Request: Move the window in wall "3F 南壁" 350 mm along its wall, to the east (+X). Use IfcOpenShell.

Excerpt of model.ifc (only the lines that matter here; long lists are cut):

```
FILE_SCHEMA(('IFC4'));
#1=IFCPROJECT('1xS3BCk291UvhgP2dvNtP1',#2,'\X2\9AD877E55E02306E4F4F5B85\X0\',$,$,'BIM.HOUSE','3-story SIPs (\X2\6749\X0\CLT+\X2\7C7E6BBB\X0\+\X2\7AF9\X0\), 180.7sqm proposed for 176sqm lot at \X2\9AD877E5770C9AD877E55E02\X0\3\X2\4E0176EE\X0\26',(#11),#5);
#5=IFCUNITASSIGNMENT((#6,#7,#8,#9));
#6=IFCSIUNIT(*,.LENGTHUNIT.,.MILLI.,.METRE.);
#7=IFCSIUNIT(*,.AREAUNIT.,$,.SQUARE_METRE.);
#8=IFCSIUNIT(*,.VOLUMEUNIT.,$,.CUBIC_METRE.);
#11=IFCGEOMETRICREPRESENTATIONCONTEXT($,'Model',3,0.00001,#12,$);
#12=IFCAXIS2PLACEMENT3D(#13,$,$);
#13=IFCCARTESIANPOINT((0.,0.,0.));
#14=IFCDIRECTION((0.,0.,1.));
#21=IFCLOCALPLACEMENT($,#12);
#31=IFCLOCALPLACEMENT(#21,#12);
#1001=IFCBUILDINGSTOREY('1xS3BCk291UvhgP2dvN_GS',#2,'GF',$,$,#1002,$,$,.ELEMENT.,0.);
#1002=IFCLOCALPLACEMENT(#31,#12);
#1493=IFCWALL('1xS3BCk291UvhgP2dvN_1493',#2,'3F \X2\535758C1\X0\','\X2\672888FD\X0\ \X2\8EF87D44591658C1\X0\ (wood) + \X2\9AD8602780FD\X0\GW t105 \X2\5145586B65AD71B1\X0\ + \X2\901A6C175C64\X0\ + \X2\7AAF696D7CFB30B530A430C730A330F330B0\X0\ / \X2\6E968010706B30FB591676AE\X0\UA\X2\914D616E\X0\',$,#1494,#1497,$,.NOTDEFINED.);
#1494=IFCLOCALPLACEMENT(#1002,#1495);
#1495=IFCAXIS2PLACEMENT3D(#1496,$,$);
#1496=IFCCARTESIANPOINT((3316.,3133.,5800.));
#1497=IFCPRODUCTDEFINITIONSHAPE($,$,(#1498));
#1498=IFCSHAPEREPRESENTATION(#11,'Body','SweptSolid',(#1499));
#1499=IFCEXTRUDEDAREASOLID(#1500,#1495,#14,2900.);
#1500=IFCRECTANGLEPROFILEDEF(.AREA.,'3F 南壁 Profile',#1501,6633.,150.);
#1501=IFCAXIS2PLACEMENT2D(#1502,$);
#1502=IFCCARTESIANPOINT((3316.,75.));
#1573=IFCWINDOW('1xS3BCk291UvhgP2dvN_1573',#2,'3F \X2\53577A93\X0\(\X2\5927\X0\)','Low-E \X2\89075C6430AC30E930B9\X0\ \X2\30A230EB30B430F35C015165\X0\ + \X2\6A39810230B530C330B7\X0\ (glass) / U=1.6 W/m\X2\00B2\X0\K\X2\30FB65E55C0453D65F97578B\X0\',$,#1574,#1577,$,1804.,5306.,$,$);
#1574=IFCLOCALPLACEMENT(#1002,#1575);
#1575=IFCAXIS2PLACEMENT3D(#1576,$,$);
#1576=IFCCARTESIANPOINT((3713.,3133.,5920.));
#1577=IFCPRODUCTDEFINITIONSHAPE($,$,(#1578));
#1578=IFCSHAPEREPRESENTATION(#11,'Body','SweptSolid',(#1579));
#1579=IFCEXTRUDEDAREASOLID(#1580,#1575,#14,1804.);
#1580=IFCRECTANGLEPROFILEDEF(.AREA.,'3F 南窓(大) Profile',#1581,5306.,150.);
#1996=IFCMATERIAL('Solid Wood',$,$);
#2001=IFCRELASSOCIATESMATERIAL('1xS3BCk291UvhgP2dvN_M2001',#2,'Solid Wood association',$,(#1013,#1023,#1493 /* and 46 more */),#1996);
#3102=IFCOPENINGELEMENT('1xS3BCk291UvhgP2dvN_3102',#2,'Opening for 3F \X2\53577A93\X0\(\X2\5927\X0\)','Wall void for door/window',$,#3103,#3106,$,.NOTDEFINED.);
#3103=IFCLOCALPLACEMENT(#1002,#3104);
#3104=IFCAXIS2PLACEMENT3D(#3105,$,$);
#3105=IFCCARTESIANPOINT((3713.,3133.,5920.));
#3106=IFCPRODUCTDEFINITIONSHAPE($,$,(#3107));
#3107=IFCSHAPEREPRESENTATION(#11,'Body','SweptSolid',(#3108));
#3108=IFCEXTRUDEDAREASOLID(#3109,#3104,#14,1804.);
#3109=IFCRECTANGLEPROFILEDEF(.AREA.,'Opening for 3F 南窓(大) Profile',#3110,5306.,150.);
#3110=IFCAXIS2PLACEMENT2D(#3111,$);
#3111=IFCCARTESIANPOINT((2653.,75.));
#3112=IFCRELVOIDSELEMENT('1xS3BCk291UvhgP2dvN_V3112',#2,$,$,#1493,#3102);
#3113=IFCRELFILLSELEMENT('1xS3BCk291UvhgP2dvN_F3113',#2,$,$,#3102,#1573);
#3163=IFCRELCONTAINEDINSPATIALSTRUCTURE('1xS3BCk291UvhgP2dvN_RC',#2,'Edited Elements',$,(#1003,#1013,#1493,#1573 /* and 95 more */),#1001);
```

```python
import ifcopenshell
import ifcopenshell.api.geometry
import ifcopenshell.util.placement
import ifcopenshell.util.unit

model = ifcopenshell.open("model.ifc")
unit_scale = ifcopenshell.util.unit.calculate_unit_scale(model)

window = model.by_id(1573)
opening = window.FillsVoids[0].RelatingOpeningElement
wall = opening.VoidsElements[0].RelatingBuildingElement

wall_matrix = ifcopenshell.util.placement.get_local_placement(wall.ObjectPlacement)
shift = wall_matrix[:3, 0] * 0.35 / unit_scale
before = ifcopenshell.util.placement.get_local_placement(window.ObjectPlacement)[:3, 3].copy()

# The window is not placed relative to its opening, so move both.
for product in (opening, window):
    matrix = ifcopenshell.util.placement.get_local_placement(product.ObjectPlacement)
    matrix[:3, 3] += shift
    ifcopenshell.api.geometry.edit_object_placement(model, product=product, matrix=matrix, is_si=False)

after = ifcopenshell.util.placement.get_local_placement(window.ObjectPlacement)[:3, 3]
print("window moved by", (after - before).round(3) + 0.0)

model.write("model_rev.ifc")
```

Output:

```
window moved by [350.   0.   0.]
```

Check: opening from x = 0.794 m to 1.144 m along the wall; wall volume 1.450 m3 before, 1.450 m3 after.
